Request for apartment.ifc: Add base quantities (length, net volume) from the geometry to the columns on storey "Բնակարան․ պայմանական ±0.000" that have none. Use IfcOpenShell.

First a look at what the model holds.

```python
import ifcopenshell
import ifcopenshell.util.element
import ifcopenshell.util.unit

model = ifcopenshell.open("apartment.ifc")
print(model.schema)
for unit_type in ("LENGTHUNIT", "AREAUNIT", "VOLUMEUNIT"):
    print(unit_type, ifcopenshell.util.unit.calculate_unit_scale(model, unit_type))
storey = next(s for s in model.by_type("IfcBuildingStorey") if s.Name == "Բնակարան․ պայմանական ±0.000")
columns = [e for e in ifcopenshell.util.element.get_decomposition(storey) if e.is_a("IfcColumn")]
for e in sorted(columns, key=lambda e: e.id()):
    print(e.id(), e.is_a(), e.Name, list(ifcopenshell.util.element.get_psets(e, qtos_only=True)), sep=" | ")
```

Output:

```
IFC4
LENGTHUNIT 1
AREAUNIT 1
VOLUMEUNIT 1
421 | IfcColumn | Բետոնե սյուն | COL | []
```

```python
import ifcopenshell
import ifcopenshell.api.pset
import ifcopenshell.geom
import ifcopenshell.util.element
import ifcopenshell.util.shape
import ifcopenshell.util.unit

model = ifcopenshell.open("apartment.ifc")
unit_scale = ifcopenshell.util.unit.calculate_unit_scale(model)
volume_scale = ifcopenshell.util.unit.calculate_unit_scale(model, "VOLUMEUNIT")
settings = ifcopenshell.geom.settings()

storey = next(s for s in model.by_type("IfcBuildingStorey") if s.Name == "Բնակարան․ պայմանական ±0.000")
columns = [e for e in ifcopenshell.util.element.get_decomposition(storey) if e.is_a("IfcColumn")]

for e in sorted(columns, key=lambda e: e.id()):
    if ifcopenshell.util.element.get_psets(e, qtos_only=True, should_inherit=False):
        continue
    # Geometry comes back in metres, in the element's own axes.
    shape = ifcopenshell.geom.create_shape(settings, e)
    values = {
        "Length": ifcopenshell.util.shape.get_z(shape.geometry) / unit_scale,
        "NetVolume": ifcopenshell.util.shape.get_volume(shape.geometry) / volume_scale,
    }
    qto = ifcopenshell.api.pset.add_qto(model, product=e, name="Qto_ColumnBaseQuantities")
    ifcopenshell.api.pset.edit_qto(model, qto=qto, properties=values)
    print(e.id(), {k: round(v, 3) for k, v in values.items()})

model.write("apartment_edited.ifc")
```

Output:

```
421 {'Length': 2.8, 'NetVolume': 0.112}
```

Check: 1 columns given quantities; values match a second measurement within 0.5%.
